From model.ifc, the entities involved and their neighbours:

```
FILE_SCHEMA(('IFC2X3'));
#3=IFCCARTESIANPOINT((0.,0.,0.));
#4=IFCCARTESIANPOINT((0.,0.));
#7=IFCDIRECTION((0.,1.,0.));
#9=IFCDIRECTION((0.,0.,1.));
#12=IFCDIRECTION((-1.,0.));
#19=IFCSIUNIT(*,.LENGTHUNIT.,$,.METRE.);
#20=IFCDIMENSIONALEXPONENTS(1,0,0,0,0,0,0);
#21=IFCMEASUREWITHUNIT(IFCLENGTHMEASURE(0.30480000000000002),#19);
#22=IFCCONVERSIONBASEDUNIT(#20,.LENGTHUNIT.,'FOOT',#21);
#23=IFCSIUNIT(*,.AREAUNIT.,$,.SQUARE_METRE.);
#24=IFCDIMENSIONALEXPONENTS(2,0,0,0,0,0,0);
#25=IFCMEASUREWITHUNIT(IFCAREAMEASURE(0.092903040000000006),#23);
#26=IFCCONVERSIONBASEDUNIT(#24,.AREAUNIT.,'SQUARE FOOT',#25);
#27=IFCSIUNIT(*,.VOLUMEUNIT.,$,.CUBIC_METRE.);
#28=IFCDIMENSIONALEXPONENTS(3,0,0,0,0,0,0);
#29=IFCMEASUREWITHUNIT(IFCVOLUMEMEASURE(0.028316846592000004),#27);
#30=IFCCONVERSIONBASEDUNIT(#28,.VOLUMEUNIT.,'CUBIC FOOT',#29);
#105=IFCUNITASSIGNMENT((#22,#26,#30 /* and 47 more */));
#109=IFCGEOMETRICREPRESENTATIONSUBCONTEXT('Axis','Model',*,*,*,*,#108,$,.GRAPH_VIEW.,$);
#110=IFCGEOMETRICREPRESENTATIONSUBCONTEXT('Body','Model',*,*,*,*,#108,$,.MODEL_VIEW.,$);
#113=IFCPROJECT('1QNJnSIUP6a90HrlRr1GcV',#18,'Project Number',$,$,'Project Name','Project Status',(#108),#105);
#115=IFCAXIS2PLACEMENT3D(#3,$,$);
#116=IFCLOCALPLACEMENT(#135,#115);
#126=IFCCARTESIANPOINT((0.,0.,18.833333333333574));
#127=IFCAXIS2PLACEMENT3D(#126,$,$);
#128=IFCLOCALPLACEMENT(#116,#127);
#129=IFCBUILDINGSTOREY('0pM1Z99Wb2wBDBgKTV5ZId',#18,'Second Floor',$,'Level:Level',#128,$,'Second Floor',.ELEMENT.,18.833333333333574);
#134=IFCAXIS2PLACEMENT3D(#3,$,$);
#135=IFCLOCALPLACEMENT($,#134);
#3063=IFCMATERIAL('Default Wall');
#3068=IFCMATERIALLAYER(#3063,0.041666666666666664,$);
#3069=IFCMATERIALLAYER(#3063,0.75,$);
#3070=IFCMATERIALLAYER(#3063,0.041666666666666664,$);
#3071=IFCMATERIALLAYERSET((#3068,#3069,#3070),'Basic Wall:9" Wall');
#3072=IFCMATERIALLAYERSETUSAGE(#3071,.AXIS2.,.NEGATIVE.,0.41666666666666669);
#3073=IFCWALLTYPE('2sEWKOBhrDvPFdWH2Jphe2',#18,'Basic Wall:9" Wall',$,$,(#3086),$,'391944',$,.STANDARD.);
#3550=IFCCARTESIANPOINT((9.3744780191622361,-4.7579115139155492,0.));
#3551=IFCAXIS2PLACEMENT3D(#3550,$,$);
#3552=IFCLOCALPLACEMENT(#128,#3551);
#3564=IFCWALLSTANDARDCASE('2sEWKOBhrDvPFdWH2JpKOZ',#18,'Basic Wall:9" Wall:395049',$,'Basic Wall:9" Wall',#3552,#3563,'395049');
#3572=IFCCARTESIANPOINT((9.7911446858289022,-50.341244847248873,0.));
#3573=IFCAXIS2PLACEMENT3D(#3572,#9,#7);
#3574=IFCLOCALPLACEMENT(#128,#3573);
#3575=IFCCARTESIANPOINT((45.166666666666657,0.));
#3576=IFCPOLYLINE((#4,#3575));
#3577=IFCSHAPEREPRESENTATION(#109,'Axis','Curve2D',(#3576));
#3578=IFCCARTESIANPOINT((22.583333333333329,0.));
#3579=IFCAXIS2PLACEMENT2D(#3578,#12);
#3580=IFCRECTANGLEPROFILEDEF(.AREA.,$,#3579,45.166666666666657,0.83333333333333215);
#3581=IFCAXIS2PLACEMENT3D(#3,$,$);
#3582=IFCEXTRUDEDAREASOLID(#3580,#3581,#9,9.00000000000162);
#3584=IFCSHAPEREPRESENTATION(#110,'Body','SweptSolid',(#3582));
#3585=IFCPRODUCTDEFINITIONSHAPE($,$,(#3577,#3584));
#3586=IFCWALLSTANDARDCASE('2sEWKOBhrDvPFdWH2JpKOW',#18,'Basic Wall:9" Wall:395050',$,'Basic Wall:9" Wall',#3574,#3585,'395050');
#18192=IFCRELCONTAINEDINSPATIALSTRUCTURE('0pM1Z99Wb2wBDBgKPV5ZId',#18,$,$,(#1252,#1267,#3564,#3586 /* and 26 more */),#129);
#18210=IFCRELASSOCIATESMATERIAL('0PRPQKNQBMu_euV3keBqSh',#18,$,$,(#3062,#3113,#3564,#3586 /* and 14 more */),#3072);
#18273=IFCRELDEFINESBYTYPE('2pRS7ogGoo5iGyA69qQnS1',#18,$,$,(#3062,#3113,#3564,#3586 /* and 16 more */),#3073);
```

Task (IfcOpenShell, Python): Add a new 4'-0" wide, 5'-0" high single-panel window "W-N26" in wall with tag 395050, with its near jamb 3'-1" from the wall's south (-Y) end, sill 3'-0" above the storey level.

```python
import numpy as np
import ifcopenshell
import ifcopenshell.api.feature
import ifcopenshell.api.geometry
import ifcopenshell.api.root
import ifcopenshell.api.spatial
import ifcopenshell.api.type
import ifcopenshell.geom
import ifcopenshell.util.element
import ifcopenshell.util.placement
import ifcopenshell.util.representation
import ifcopenshell.util.shape
import ifcopenshell.util.unit

model = ifcopenshell.open("model.ifc")
unit_scale = ifcopenshell.util.unit.calculate_unit_scale(model)
settings = ifcopenshell.geom.settings()


def volume(element):
    """Net volume in cubic metres, openings subtracted."""
    shape = ifcopenshell.geom.create_shape(settings, element)
    return ifcopenshell.util.shape.get_volume(shape.geometry)


wall = model.by_id(3586)
storey = ifcopenshell.util.element.get_container(wall, ifc_class="IfcBuildingStorey")
context = ifcopenshell.util.representation.get_context(model, "Model", "Body", "MODEL_VIEW")
before = volume(wall)

width, height, from_end, sill = 1.2192, 1.524, 0.9398, 0.9144  # metres

# The wall runs along its own X axis, and the end named is its -X end.
wall_shape = ifcopenshell.geom.create_shape(settings, wall)
x, y, z = ifcopenshell.util.shape.get_vertices(wall_shape.geometry).T
start = x.min() + from_end
face, thickness = float(y.min()), float(y.max() - y.min())
wall_matrix = ifcopenshell.util.placement.get_local_placement(wall.ObjectPlacement)
level = ifcopenshell.util.placement.get_local_placement(storey.ObjectPlacement)[2, 3]


def in_wall(x, y):
    """Placement at x, y metres in the wall's axes, at sill height."""
    matrix = wall_matrix.copy()
    matrix[:, 3] = wall_matrix @ np.array([x / unit_scale, y / unit_scale, 0.0, 1.0])
    matrix[2, 3] = level + sill / unit_scale
    return matrix


# Opening: a box that overshoots both wall faces by 50 mm.
opening = ifcopenshell.api.root.create_entity(model, ifc_class="IfcOpeningElement")
box = ifcopenshell.api.geometry.add_wall_representation(
    model, context=context, length=width, height=height, thickness=thickness + 0.1
)
ifcopenshell.api.geometry.assign_representation(model, product=opening, representation=box)
ifcopenshell.api.geometry.edit_object_placement(model, product=opening, matrix=in_wall(start, face - 0.05), is_si=False)
ifcopenshell.api.feature.add_feature(model, feature=opening, element=wall)

window = ifcopenshell.api.root.create_entity(model, ifc_class="IfcWindow", name="W-N26")
window.OverallWidth, window.OverallHeight = width / unit_scale, height / unit_scale
body = ifcopenshell.api.geometry.add_window_representation(
    model,
    context=context,
    overall_width=window.OverallWidth,
    overall_height=window.OverallHeight,
    partition_type="SINGLE_PANEL",
)
ifcopenshell.api.geometry.assign_representation(model, product=window, representation=body)
ifcopenshell.api.spatial.assign_container(model, products=[window], relating_structure=storey)
fills = ifcopenshell.api.feature.add_filling(model, opening=opening, element=window)
fills.OwnerHistory = window.OwnerHistory  # required in IFC2X3

# IFC2X3 keeps the operation on the window style.
style = ifcopenshell.api.root.create_entity(model, ifc_class="IfcWindowStyle", name="W-N26")
style.OperationType, style.ConstructionType = "SINGLE_PANEL", "NOTDEFINED"
style.ParameterTakesPrecedence = style.Sizeable = False
ifcopenshell.api.type.assign_type(model, related_objects=[window], relating_type=style)

# Centre the window in the wall's thickness.
ifcopenshell.api.geometry.edit_object_placement(model, product=window, matrix=in_wall(start, face), is_si=False)
window_shape = ifcopenshell.geom.create_shape(settings, window)
depth = ifcopenshell.util.shape.get_vertices(window_shape.geometry)[:, 1]
offset = face + thickness / 2 - (depth.min() + depth.max()) / 2
ifcopenshell.api.geometry.edit_object_placement(model, product=window, matrix=in_wall(start, offset), is_si=False)

after = volume(wall)

print(f"wall volume {before:.3f} -> {after:.3f} m3")

model.write("model_v2.ifc")
```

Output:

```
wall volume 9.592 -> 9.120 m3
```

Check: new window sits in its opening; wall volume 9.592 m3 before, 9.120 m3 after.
